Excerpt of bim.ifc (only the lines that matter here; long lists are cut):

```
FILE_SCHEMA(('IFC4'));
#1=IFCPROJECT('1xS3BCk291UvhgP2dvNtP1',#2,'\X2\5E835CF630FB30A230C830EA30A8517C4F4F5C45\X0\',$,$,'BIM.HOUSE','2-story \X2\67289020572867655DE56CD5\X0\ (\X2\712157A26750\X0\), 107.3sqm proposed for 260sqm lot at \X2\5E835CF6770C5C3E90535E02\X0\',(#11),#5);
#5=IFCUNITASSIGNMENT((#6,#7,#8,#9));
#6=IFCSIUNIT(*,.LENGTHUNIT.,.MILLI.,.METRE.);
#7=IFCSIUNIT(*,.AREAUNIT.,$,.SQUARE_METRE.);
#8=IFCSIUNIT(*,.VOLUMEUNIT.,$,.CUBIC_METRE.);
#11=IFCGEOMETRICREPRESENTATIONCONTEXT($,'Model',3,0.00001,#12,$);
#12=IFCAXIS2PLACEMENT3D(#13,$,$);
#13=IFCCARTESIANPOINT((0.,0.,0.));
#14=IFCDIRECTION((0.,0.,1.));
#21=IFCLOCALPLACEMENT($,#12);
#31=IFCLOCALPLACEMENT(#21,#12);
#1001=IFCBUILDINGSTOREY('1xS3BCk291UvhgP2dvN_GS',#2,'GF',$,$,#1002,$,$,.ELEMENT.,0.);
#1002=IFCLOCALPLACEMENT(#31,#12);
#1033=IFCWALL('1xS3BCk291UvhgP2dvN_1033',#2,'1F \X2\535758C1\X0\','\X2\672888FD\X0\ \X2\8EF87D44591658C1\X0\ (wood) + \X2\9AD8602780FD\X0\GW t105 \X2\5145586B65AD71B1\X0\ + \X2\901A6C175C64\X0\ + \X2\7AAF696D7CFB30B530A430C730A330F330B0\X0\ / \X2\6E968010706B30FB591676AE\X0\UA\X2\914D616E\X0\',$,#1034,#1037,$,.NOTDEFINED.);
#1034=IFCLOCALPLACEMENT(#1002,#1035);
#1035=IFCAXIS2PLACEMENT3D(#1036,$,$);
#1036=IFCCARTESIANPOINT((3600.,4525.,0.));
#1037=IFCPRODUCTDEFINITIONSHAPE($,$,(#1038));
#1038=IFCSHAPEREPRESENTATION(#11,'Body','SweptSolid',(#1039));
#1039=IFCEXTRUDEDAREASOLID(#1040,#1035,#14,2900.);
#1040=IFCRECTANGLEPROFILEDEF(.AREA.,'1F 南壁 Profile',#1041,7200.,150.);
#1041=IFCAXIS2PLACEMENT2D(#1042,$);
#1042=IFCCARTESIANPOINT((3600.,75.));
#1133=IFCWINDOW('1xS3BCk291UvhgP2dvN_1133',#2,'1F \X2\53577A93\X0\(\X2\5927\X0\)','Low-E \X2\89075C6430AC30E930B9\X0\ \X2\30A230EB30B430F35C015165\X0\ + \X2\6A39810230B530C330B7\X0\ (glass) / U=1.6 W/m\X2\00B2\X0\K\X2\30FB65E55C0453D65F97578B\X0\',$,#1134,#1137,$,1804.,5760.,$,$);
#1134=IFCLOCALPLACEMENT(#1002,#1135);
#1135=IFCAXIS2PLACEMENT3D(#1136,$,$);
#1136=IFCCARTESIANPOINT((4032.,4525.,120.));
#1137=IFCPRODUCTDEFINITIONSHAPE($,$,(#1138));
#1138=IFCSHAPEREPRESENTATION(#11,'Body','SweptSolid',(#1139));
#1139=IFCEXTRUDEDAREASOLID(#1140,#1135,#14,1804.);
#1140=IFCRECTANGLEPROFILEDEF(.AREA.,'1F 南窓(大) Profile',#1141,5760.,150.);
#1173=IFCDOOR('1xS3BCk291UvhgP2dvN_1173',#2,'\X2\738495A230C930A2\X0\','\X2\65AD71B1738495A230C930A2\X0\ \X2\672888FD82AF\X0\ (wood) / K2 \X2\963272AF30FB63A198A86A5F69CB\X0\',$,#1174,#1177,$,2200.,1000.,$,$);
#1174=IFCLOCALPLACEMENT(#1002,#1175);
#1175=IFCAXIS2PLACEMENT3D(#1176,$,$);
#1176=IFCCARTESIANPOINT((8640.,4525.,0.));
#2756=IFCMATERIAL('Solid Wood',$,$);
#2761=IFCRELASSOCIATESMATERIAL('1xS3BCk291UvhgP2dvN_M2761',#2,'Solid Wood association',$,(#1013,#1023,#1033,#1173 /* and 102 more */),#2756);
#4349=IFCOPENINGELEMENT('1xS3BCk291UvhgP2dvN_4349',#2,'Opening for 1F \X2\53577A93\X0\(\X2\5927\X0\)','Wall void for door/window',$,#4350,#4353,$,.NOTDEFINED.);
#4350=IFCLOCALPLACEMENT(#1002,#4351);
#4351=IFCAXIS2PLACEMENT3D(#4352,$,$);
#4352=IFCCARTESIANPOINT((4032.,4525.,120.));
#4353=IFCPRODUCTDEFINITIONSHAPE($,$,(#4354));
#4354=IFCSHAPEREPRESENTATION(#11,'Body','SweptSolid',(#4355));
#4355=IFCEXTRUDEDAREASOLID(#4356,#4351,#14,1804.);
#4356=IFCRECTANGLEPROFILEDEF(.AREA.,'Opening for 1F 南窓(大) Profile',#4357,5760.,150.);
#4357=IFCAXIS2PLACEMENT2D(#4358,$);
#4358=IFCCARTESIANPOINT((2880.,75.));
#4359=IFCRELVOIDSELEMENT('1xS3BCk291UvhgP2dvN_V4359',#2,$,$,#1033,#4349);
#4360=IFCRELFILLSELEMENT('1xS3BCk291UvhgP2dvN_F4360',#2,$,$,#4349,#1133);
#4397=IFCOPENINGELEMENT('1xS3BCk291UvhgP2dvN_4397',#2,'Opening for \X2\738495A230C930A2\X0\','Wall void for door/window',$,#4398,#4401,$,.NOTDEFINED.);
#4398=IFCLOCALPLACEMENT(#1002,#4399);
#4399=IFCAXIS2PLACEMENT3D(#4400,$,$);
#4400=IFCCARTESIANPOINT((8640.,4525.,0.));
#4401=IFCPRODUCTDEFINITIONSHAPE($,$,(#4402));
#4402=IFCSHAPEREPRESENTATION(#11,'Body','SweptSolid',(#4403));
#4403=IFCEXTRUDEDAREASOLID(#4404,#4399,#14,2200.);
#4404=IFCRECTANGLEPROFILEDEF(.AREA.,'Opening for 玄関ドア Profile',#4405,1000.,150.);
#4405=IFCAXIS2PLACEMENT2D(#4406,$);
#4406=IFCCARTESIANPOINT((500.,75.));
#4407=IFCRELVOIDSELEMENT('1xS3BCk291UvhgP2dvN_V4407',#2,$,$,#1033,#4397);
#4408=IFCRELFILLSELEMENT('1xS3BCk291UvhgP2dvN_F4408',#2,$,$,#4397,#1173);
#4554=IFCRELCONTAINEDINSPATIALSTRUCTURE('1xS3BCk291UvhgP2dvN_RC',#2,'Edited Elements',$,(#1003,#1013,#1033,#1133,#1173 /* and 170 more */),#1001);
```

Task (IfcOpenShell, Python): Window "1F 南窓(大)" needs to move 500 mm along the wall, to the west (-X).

```python
import ifcopenshell
import ifcopenshell.api.geometry
import ifcopenshell.util.placement
import ifcopenshell.util.unit

model = ifcopenshell.open("bim.ifc")
unit_scale = ifcopenshell.util.unit.calculate_unit_scale(model)

window = model.by_guid("1xS3BCk291UvhgP2dvN_1133")
opening = window.FillsVoids[0].RelatingOpeningElement
wall = opening.VoidsElements[0].RelatingBuildingElement

wall_matrix = ifcopenshell.util.placement.get_local_placement(wall.ObjectPlacement)
shift = wall_matrix[:3, 0] * -0.5 / unit_scale
before = ifcopenshell.util.placement.get_local_placement(window.ObjectPlacement)[:3, 3].copy()

# The window is not placed relative to its opening, so move both.
for product in (opening, window):
    matrix = ifcopenshell.util.placement.get_local_placement(product.ObjectPlacement)
    matrix[:3, 3] += shift
    ifcopenshell.api.geometry.edit_object_placement(model, product=product, matrix=matrix, is_si=False)

after = ifcopenshell.util.placement.get_local_placement(window.ObjectPlacement)[:3, 3]
print("window moved by", (after - before).round(3) + 0.0)

model.write("bim_v2.ifc")
```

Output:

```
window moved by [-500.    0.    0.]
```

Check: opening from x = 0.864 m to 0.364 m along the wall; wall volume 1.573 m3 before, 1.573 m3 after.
